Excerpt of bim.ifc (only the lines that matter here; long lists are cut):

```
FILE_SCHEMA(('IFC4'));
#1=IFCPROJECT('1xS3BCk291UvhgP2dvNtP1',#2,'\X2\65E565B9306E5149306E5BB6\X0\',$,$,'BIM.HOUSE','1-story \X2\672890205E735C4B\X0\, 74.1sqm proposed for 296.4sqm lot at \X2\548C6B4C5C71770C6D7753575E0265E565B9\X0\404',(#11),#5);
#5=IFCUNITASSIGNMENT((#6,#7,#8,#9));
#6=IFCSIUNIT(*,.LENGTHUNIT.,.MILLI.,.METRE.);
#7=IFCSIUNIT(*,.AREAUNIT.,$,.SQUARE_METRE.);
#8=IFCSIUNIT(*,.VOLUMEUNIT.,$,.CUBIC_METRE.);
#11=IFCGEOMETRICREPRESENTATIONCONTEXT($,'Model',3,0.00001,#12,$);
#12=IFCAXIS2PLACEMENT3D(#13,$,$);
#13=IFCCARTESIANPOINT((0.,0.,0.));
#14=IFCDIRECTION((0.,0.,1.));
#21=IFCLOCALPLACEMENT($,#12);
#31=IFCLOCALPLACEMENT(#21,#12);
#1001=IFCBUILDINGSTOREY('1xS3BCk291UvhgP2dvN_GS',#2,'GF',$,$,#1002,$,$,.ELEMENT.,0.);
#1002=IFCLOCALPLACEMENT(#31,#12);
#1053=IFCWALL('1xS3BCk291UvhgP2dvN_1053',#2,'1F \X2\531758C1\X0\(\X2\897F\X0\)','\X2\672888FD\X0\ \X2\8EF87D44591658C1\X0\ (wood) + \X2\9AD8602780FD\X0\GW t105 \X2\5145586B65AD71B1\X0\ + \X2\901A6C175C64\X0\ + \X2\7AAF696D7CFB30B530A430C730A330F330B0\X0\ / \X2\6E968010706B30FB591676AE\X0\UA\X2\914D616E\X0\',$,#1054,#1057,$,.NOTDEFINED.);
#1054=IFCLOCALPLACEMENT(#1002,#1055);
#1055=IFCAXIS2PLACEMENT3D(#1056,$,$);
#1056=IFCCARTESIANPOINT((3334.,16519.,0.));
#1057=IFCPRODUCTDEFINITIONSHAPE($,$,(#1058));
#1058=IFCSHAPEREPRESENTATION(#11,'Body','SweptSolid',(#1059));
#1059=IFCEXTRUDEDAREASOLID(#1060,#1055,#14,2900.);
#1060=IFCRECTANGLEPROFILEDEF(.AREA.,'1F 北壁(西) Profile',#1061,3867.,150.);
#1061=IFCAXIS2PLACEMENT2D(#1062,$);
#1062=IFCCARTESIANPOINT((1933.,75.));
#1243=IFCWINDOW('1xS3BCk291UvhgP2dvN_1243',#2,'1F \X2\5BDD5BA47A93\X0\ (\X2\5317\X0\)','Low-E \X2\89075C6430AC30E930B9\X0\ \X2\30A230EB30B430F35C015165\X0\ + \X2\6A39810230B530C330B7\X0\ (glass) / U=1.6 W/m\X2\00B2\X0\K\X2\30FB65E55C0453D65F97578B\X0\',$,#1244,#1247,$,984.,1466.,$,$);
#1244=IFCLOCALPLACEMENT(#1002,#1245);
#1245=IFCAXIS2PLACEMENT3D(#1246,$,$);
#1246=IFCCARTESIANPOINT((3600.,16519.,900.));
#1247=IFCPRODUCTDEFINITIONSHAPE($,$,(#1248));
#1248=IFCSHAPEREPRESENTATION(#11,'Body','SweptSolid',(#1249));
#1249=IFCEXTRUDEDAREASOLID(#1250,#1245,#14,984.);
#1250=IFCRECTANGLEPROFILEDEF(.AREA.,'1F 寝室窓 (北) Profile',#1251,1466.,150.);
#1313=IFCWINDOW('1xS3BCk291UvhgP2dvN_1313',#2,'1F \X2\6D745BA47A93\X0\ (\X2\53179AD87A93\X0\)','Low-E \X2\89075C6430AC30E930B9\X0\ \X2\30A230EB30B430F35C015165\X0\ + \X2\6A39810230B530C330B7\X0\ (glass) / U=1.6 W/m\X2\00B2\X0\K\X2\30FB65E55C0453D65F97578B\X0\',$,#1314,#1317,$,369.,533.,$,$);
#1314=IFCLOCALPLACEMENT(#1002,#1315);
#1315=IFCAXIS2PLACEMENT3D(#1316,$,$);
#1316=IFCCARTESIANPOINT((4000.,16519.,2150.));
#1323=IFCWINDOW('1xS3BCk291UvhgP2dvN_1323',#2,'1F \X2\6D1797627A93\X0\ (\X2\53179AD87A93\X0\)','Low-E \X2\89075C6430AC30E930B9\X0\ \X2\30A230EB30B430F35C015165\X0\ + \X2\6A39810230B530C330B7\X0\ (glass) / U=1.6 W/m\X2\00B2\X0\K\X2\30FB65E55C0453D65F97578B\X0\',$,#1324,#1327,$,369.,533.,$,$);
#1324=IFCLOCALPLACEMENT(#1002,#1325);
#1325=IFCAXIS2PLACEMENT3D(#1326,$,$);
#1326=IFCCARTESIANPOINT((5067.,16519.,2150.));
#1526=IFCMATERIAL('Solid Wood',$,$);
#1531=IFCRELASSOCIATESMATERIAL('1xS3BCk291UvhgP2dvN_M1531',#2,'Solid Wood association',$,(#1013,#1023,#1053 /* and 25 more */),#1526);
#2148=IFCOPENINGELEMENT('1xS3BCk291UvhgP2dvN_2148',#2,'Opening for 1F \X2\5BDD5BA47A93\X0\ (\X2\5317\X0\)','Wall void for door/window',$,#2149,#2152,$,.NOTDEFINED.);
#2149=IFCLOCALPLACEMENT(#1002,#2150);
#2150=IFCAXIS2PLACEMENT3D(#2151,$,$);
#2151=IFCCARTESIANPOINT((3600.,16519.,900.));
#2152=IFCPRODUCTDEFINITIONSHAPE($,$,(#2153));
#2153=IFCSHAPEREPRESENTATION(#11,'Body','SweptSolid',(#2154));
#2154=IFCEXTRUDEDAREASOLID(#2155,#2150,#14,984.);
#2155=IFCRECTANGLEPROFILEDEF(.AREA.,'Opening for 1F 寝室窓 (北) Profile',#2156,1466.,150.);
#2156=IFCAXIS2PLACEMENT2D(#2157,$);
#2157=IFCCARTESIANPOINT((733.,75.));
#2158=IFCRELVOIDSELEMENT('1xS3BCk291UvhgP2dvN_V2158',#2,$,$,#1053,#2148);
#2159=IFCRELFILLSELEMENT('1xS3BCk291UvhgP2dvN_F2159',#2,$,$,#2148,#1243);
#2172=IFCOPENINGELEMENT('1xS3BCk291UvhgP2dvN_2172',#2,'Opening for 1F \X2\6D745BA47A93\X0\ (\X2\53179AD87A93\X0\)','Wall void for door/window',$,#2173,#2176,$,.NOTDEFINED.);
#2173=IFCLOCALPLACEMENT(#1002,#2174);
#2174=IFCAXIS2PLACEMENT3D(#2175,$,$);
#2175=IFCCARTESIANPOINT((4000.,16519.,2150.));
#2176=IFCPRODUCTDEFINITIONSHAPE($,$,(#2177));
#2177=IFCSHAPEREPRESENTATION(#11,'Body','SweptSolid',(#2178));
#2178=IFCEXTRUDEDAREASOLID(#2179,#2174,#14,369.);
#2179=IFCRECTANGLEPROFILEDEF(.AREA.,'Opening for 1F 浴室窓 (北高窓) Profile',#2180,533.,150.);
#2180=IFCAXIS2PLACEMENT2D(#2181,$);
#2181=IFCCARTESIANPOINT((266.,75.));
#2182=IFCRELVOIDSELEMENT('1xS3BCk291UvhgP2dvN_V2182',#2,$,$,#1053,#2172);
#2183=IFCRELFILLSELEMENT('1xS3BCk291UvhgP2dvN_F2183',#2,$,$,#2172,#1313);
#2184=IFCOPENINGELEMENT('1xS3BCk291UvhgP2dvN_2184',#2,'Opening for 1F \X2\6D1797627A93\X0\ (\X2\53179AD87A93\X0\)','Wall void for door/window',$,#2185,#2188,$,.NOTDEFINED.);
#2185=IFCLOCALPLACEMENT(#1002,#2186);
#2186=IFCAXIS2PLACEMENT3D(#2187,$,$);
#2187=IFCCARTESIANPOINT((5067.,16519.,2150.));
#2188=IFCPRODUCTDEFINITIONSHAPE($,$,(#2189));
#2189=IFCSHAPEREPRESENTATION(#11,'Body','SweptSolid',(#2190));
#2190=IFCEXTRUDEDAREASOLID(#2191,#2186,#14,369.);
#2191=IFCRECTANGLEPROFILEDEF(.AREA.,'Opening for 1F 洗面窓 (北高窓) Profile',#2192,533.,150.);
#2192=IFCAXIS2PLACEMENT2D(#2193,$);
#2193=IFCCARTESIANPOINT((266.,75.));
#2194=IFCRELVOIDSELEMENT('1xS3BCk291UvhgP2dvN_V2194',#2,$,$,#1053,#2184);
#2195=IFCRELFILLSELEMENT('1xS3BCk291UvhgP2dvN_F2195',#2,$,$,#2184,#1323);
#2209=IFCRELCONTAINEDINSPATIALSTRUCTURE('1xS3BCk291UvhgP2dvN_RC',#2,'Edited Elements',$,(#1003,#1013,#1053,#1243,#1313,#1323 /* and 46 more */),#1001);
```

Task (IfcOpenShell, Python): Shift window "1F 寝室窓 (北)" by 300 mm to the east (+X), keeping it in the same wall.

```python
import ifcopenshell
import ifcopenshell.api.geometry
import ifcopenshell.util.placement

model = ifcopenshell.open("bim.ifc")

window = model.by_id(1243)
opening = window.FillsVoids[0].RelatingOpeningElement
wall = opening.VoidsElements[0].RelatingBuildingElement

wall_matrix = ifcopenshell.util.placement.get_local_placement(wall.ObjectPlacement)
shift = wall_matrix[:3, 0] * 300.0
before = ifcopenshell.util.placement.get_local_placement(window.ObjectPlacement)[:3, 3].copy()

# The window is not placed relative to its opening, so move both.
for product in (opening, window):
    matrix = ifcopenshell.util.placement.get_local_placement(product.ObjectPlacement)
    matrix[:3, 3] += shift
    ifcopenshell.api.geometry.edit_object_placement(model, product=product, matrix=matrix, is_si=False)

after = ifcopenshell.util.placement.get_local_placement(window.ObjectPlacement)[:3, 3]
print("window moved by", (after - before).round(3) + 0.0)

model.write("bim-out.ifc")
```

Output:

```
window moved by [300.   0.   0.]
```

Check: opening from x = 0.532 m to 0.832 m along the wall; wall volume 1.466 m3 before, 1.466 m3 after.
